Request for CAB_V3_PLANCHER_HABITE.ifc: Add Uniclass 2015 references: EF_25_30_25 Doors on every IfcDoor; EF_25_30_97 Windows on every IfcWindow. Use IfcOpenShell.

First a look at what the model holds.

```python
import ifcopenshell

model = ifcopenshell.open("CAB_V3_PLANCHER_HABITE.ifc")
print(model.schema)
print("classifications:", [c.Name for c in model.by_type("IfcClassification")])
for ifc_class in ("IfcDoor", "IfcRoof", "IfcStair", "IfcWall", "IfcWindow"):
    print(ifc_class, len(model.by_type(ifc_class)))
```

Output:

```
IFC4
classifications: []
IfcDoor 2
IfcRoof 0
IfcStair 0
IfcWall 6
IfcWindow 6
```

```python
import ifcopenshell
import ifcopenshell.api.classification

model = ifcopenshell.open("CAB_V3_PLANCHER_HABITE.ifc")

system = ifcopenshell.api.classification.add_classification(model, classification="Uniclass 2015")

codes = {
    "IfcDoor": ("EF_25_30_25", "Doors"),
    "IfcWindow": ("EF_25_30_97", "Windows"),
}
for ifc_class, (code, name) in codes.items():
    products = model.by_type(ifc_class)
    ifcopenshell.api.classification.add_reference(
        model, products=products, classification=system, identification=code, name=name
    )
    print(code, len(products))

model.write("CAB_V3_PLANCHER_HABITE_edited.ifc")
```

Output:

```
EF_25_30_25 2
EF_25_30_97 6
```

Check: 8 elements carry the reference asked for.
